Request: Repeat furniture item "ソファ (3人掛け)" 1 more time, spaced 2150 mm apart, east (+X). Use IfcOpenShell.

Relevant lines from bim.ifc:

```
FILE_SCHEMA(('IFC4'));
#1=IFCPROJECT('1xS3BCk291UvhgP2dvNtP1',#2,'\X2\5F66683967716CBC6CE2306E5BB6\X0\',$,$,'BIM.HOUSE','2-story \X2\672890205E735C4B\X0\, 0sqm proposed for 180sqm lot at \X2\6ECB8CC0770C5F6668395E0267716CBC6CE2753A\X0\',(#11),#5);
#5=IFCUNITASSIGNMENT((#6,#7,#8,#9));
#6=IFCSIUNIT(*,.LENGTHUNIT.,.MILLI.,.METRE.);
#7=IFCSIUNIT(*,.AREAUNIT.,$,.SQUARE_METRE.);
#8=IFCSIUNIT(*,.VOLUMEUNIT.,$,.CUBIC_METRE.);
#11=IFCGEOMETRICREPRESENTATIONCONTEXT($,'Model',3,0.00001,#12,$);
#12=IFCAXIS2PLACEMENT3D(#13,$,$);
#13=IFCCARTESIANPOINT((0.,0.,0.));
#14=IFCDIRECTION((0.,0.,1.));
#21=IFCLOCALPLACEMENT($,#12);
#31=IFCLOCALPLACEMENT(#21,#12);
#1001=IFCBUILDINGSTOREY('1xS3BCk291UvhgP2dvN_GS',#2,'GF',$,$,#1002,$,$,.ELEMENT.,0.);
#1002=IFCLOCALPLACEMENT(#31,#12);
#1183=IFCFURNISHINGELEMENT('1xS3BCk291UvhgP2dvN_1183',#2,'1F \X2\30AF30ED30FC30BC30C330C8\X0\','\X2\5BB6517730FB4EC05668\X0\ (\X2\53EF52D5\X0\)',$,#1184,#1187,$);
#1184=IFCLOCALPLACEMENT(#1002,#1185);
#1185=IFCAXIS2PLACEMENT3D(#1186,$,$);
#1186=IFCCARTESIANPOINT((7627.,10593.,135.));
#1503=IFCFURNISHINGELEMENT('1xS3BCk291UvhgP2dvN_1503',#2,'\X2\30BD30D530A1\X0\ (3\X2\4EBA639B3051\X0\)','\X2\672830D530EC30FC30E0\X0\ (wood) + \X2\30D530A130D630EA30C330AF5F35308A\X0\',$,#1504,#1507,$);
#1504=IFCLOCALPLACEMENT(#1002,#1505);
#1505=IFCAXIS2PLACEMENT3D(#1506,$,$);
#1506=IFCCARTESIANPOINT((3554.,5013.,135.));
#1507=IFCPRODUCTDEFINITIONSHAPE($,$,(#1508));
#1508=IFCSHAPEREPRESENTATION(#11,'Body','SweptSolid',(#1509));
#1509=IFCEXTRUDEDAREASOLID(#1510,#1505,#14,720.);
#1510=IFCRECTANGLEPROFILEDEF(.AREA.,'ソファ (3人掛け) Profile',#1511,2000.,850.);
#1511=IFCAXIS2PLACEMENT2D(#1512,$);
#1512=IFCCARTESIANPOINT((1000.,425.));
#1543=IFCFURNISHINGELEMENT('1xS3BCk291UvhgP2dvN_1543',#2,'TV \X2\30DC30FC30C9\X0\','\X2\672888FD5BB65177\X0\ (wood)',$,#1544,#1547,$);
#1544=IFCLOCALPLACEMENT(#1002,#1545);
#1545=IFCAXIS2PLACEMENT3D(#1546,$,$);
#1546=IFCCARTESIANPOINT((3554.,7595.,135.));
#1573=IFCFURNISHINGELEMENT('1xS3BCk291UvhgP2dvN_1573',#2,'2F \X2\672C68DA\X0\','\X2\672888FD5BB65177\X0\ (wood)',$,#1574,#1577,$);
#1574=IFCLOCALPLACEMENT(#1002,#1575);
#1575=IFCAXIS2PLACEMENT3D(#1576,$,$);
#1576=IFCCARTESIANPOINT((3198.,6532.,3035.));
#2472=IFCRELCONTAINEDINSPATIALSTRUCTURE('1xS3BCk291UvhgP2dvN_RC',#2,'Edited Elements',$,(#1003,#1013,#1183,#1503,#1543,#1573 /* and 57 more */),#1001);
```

```python
import numpy as np
import ifcopenshell
import ifcopenshell.api.geometry
import ifcopenshell.api.root
import ifcopenshell.util.element
import ifcopenshell.util.placement
import ifcopenshell.util.unit

model = ifcopenshell.open("bim.ifc")
unit_scale = ifcopenshell.util.unit.calculate_unit_scale(model)


def reuse_history(source, copy):
    """copy_class also copies each property set's owner history, people and application; keep the originals."""
    for rel in copy.IsDefinedBy:
        if rel.is_a("IfcRelDefinesByProperties") and (history := rel.RelatingPropertyDefinition.OwnerHistory):
            rel.RelatingPropertyDefinition.OwnerHistory = source.OwnerHistory
            ifcopenshell.util.element.remove_deep2(model, history)


source = model.by_guid("1xS3BCk291UvhgP2dvN_1503")
base = ifcopenshell.util.placement.get_local_placement(source.ObjectPlacement)
step = np.array([1.0, 0.0, 0.0]) * 2.15 / unit_scale

for i in range(1, 2):
    copy = ifcopenshell.api.root.copy_class(model, product=source)
    copy.Representation = ifcopenshell.util.element.copy_deep(
        model, source.Representation, exclude=["IfcGeometricRepresentationContext", "IfcRepresentationMap"]
    )
    reuse_history(source, copy)
    matrix = base.copy()
    matrix[:3, 3] += i * step
    print("added at", matrix[:3, 3].round(3) + 0.0)
    ifcopenshell.api.geometry.edit_object_placement(model, product=copy, matrix=matrix, is_si=False)

model.write("bim_rev.ifc")
```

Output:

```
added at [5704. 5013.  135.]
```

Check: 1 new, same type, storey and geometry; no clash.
